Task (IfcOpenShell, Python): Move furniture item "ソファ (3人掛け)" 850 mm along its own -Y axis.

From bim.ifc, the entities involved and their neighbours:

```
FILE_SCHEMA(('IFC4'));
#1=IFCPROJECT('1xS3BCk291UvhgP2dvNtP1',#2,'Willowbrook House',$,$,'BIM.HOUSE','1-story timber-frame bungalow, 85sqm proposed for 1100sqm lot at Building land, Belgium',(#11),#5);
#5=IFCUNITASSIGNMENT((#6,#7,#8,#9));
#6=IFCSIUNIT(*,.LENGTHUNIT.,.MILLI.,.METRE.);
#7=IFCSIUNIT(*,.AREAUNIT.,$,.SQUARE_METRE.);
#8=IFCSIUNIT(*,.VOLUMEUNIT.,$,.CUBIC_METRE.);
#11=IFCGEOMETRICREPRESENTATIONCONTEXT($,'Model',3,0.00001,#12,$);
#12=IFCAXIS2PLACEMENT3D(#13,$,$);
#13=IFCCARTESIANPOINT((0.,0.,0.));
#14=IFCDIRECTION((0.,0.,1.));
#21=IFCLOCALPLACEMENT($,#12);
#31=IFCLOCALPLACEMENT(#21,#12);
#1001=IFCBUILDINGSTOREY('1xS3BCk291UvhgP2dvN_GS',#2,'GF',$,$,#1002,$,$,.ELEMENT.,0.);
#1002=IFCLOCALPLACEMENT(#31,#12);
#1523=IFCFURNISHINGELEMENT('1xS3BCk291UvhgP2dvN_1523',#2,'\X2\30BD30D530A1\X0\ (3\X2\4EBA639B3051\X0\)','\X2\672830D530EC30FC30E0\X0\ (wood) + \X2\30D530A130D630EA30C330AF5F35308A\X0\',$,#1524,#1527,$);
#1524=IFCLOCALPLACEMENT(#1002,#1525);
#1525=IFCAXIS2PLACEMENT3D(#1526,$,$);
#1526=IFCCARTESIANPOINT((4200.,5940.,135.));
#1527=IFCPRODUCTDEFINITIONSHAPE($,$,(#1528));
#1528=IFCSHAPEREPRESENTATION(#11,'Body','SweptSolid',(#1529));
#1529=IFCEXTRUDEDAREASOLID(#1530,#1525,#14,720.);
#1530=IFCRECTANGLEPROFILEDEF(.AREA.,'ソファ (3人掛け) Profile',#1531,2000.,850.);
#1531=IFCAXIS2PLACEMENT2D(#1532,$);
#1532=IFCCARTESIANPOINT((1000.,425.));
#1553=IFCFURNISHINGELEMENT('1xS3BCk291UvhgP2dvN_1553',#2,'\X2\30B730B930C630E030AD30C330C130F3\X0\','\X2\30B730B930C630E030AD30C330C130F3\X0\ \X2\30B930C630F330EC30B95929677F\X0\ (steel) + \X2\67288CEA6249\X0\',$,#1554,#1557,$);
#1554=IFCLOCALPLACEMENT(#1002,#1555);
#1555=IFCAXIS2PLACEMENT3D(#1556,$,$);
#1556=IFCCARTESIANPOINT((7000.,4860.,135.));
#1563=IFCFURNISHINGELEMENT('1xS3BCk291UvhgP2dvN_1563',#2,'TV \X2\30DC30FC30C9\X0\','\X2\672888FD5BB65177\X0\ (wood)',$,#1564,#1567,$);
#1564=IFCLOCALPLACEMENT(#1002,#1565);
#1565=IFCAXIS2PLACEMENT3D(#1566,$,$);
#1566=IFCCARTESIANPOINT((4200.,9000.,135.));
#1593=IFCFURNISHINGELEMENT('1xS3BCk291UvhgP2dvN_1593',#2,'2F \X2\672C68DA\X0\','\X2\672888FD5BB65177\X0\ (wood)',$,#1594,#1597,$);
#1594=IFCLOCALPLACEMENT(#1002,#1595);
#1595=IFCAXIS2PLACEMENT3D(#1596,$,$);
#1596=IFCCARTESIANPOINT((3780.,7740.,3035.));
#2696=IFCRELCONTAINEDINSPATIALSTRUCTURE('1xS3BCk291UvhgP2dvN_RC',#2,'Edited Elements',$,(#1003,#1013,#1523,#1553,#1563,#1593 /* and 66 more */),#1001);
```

```python
import ifcopenshell
import ifcopenshell.api.geometry
import ifcopenshell.util.placement
import ifcopenshell.util.unit

model = ifcopenshell.open("bim.ifc")
unit_scale = ifcopenshell.util.unit.calculate_unit_scale(model)

item = model.by_id(1523)
matrix = ifcopenshell.util.placement.get_local_placement(item.ObjectPlacement)
matrix[:3, 3] -= matrix[:3, 1] * 0.85 / unit_scale
ifcopenshell.api.geometry.edit_object_placement(model, product=item, matrix=matrix, is_si=False)

print(ifcopenshell.util.placement.get_local_placement(item.ObjectPlacement).round(3) + 0.0)

model.write("bim_v2.ifc")
```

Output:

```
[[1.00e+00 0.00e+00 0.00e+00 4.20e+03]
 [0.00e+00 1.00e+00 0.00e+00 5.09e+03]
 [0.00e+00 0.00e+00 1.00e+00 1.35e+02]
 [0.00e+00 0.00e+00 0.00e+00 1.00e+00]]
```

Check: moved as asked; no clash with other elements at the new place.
